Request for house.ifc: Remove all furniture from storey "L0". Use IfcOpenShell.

First a look at what the model holds.

```python
import ifcopenshell
import ifcopenshell.util.element

model = ifcopenshell.open("house.ifc")
print(model.schema)
storey = next(s for s in model.by_type("IfcBuildingStorey") if s.Name == "L0")
furniture = [e for e in ifcopenshell.util.element.get_decomposition(storey) if e.is_a("IfcFurnishingElement")]
seen = {}
for e in furniture:
    element_type = ifcopenshell.util.element.get_type(e)
    name = element_type.Name if element_type not in (None, e) else None
    seen[name] = seen.get(name, 0) + 1
for name, count in sorted(seen.items(), key=str):
    print(count, "x", name)
```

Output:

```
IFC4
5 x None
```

```python
import ifcopenshell
import ifcopenshell.api.root
import ifcopenshell.util.element

model = ifcopenshell.open("house.ifc")

storey = next(s for s in model.by_type("IfcBuildingStorey") if s.Name == "L0")
furniture = [e for e in ifcopenshell.util.element.get_decomposition(storey) if e.is_a("IfcFurnishingElement")]

for e in furniture:
    ifcopenshell.api.root.remove_product(model, product=e)
print(len(furniture), "removed")

model.write("house-out.ifc")
```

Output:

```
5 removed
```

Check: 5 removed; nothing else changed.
